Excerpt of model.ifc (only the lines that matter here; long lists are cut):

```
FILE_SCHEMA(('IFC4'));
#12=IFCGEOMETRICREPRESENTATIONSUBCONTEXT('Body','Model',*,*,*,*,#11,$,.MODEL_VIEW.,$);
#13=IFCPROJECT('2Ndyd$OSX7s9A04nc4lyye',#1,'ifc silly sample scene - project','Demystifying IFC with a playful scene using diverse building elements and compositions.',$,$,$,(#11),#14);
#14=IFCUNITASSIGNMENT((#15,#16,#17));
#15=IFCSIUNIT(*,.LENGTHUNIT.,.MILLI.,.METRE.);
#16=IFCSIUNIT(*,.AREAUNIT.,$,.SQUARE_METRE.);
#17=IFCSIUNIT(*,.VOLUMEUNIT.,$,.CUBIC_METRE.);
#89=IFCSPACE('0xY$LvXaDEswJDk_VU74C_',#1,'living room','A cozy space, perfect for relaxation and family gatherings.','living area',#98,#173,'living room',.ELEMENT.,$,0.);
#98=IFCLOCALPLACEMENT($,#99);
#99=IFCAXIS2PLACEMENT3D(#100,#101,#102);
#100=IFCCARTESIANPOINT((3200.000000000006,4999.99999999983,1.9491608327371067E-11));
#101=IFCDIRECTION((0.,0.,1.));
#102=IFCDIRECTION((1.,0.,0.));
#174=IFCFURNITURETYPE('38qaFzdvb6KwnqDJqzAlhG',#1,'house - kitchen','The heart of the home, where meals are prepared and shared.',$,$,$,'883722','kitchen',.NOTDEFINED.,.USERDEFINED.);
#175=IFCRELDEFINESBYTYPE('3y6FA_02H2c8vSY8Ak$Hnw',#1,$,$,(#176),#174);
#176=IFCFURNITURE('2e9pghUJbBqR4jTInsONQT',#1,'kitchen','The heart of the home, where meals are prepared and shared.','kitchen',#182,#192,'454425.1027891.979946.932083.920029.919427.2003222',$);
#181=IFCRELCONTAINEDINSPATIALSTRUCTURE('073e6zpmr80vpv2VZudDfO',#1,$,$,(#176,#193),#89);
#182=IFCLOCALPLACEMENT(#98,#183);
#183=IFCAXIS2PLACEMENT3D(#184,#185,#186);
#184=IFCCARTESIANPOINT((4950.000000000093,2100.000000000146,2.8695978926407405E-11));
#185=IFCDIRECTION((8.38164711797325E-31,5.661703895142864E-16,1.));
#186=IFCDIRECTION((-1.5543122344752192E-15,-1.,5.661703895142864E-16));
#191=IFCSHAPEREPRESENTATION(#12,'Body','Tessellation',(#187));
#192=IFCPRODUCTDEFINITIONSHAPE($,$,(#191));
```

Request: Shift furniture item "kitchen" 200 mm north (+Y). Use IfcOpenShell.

```python
import ifcopenshell
import ifcopenshell.api.geometry
import ifcopenshell.util.placement

model = ifcopenshell.open("model.ifc")

item = model.by_id(176)
matrix = ifcopenshell.util.placement.get_local_placement(item.ObjectPlacement)
matrix[1, 3] += 200.0
ifcopenshell.api.geometry.edit_object_placement(model, product=item, matrix=matrix, is_si=False)

print(ifcopenshell.util.placement.get_local_placement(item.ObjectPlacement).round(3) + 0.0)

model.write("model_rev.ifc")
```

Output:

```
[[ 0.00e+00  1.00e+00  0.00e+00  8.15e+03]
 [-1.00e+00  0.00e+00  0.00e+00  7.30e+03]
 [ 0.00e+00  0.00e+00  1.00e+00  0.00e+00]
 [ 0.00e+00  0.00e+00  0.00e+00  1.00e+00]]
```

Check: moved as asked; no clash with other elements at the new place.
